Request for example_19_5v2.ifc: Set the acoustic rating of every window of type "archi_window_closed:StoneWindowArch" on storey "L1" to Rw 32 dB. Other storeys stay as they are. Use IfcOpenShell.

First a look at what the model holds.

```python
import ifcopenshell
import ifcopenshell.util.element

model = ifcopenshell.open("example_19_5v2.ifc")
print(model.schema)
storey = next(s for s in model.by_type("IfcBuildingStorey") if s.Name == "L1")
windows = [e for e in ifcopenshell.util.element.get_decomposition(storey) if e.is_a("IfcWindow")]
seen = {}
for e in windows:
    element_type = ifcopenshell.util.element.get_type(e)
    key = (element_type.Name if element_type != e and element_type else None, ifcopenshell.util.element.get_pset(e, "Pset_WindowCommon", "AcousticRating"))
    seen[key] = seen.get(key, 0) + 1
for (name, value), count in sorted(seen.items(), key=str):
    print(count, "x", name, "|", value)
```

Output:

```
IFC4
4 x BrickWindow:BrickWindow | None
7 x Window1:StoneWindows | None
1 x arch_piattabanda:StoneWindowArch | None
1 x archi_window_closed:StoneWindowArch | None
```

```python
import ifcopenshell
import ifcopenshell.api.pset
import ifcopenshell.util.element

model = ifcopenshell.open("example_19_5v2.ifc")

storey = next(s for s in model.by_type("IfcBuildingStorey") if s.Name == "L1")
windows = [e for e in ifcopenshell.util.element.get_decomposition(storey) if e.is_a("IfcWindow")]

count = 0
for e in windows:
    element_type = ifcopenshell.util.element.get_type(e)
    if element_type in (None, e) or element_type.Name != "archi_window_closed:StoneWindowArch":
        continue
    # add_pset returns the element's existing set when there is one.
    pset = ifcopenshell.api.pset.add_pset(model, product=e, name="Pset_WindowCommon")
    ifcopenshell.api.pset.edit_pset(model, pset=pset, properties={"AcousticRating": "Rw 32 dB"})
    count += 1

print(count, "windows updated")

model.write("example_19_5v2_updated.ifc")
```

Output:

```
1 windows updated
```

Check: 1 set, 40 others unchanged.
